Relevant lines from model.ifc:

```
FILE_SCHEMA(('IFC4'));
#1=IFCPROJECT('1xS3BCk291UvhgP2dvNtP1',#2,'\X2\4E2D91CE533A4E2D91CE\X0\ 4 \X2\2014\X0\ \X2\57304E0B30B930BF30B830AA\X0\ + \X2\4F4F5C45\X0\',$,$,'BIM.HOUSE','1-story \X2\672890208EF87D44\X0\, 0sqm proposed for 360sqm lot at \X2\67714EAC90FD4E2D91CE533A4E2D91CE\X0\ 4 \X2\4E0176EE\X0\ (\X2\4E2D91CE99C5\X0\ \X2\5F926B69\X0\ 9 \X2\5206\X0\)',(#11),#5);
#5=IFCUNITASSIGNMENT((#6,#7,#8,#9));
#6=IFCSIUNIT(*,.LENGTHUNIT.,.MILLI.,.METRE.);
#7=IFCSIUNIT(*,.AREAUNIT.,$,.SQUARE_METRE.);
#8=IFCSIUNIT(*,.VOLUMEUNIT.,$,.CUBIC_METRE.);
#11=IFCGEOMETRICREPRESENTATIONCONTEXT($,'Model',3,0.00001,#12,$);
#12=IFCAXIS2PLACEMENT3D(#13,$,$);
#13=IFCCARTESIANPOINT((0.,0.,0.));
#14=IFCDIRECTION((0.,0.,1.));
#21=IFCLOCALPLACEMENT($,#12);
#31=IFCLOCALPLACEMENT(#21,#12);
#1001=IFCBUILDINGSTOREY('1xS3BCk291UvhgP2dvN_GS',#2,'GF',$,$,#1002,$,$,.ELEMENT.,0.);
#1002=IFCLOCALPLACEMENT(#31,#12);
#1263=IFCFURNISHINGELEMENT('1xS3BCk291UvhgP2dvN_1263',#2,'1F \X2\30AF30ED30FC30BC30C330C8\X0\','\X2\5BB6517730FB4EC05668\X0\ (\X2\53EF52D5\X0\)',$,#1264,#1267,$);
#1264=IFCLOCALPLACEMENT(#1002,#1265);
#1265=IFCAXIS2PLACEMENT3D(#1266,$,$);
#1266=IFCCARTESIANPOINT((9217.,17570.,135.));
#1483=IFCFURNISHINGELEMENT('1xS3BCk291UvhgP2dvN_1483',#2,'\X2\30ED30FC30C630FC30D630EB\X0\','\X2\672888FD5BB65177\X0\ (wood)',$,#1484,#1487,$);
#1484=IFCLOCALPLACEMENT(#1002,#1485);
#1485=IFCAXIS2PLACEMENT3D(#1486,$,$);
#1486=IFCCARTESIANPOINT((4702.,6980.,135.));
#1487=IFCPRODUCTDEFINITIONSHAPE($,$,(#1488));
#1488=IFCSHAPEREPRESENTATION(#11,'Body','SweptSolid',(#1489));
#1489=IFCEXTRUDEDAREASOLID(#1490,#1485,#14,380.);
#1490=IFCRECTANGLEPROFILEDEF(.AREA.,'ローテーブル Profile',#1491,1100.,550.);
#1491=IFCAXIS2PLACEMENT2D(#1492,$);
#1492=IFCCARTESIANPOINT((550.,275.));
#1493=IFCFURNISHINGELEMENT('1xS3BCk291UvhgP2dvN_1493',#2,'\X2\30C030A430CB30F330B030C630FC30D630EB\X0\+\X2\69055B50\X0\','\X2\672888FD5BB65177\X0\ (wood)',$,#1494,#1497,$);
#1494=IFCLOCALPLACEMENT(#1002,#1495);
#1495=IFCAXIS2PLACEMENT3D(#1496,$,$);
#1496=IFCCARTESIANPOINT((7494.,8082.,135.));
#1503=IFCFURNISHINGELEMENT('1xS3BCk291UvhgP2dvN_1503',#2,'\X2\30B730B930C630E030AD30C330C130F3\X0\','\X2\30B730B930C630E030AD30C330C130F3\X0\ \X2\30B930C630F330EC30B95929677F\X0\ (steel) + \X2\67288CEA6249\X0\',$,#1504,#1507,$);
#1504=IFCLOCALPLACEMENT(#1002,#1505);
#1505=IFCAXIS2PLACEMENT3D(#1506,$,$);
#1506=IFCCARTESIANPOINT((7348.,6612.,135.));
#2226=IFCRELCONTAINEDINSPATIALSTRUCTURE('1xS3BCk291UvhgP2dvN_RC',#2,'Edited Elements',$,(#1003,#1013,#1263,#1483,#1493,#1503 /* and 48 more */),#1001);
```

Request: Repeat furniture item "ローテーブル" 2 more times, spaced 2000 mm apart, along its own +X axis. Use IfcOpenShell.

```python
import ifcopenshell
import ifcopenshell.api.geometry
import ifcopenshell.api.root
import ifcopenshell.util.element
import ifcopenshell.util.placement

model = ifcopenshell.open("model.ifc")


def reuse_history(source, copy):
    """copy_class also copies each property set's owner history, people and application; keep the originals."""
    for rel in copy.IsDefinedBy:
        if rel.is_a("IfcRelDefinesByProperties") and (history := rel.RelatingPropertyDefinition.OwnerHistory):
            rel.RelatingPropertyDefinition.OwnerHistory = source.OwnerHistory
            ifcopenshell.util.element.remove_deep2(model, history)


source = model.by_guid("1xS3BCk291UvhgP2dvN_1483")
base = ifcopenshell.util.placement.get_local_placement(source.ObjectPlacement)
step = base[:3, 0] * 2000.0

for i in range(1, 3):
    copy = ifcopenshell.api.root.copy_class(model, product=source)
    copy.Representation = ifcopenshell.util.element.copy_deep(
        model, source.Representation, exclude=["IfcGeometricRepresentationContext", "IfcRepresentationMap"]
    )
    reuse_history(source, copy)
    matrix = base.copy()
    matrix[:3, 3] += i * step
    print("added at", matrix[:3, 3].round(3) + 0.0)
    ifcopenshell.api.geometry.edit_object_placement(model, product=copy, matrix=matrix, is_si=False)

model.write("model_rev.ifc")
```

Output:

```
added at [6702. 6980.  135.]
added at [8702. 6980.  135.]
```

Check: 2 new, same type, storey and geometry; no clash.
